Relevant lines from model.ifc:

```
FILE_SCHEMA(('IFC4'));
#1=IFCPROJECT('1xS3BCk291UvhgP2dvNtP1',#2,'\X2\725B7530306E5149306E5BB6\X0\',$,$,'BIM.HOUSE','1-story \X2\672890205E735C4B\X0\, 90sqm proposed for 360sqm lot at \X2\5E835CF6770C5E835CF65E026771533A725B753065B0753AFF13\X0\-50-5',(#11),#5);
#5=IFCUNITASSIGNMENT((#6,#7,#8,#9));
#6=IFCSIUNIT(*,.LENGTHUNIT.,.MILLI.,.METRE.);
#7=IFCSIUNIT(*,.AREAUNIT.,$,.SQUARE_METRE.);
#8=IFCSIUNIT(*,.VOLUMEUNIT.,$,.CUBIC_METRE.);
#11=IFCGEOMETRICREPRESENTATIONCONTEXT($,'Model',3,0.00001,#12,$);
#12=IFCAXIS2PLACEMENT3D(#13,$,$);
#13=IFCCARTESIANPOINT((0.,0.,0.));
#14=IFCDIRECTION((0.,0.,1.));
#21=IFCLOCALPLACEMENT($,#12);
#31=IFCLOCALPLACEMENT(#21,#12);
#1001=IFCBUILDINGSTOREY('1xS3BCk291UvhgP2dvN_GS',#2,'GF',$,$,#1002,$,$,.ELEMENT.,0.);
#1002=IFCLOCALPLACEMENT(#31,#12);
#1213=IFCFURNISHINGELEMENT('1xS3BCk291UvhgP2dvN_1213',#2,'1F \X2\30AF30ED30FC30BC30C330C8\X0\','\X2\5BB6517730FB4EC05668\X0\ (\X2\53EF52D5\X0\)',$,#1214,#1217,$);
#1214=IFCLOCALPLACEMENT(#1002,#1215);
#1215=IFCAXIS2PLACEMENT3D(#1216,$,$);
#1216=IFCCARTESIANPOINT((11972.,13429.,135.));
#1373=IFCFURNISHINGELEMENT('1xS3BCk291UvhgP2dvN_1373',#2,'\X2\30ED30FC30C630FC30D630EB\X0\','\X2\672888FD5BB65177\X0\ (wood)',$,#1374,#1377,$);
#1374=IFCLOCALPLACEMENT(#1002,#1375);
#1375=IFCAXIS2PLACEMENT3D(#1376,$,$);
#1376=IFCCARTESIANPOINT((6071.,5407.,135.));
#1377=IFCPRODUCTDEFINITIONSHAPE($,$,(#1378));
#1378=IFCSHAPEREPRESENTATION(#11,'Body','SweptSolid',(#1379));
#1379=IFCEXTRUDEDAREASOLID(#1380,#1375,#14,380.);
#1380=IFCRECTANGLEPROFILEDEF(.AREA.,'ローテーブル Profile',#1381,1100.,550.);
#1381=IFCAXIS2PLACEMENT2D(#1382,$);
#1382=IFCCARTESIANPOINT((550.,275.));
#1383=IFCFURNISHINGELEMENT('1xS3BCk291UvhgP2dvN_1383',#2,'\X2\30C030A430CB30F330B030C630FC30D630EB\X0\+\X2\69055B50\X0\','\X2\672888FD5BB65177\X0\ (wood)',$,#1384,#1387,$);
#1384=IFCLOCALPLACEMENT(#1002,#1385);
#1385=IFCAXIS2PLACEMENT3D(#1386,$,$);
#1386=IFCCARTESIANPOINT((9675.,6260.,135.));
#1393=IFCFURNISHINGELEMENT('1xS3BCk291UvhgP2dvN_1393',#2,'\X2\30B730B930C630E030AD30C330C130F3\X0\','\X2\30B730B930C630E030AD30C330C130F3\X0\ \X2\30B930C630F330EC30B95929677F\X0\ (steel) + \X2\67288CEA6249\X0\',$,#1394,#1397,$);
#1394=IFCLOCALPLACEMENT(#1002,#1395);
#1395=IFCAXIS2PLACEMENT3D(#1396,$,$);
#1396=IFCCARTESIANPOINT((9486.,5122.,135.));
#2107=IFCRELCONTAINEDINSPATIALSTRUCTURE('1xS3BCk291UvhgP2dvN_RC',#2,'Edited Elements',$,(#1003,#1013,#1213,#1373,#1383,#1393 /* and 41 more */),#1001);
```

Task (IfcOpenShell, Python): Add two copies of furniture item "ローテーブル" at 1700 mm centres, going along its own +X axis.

```python
import ifcopenshell
import ifcopenshell.api.geometry
import ifcopenshell.api.root
import ifcopenshell.util.element
import ifcopenshell.util.placement
import ifcopenshell.util.unit

model = ifcopenshell.open("model.ifc")
unit_scale = ifcopenshell.util.unit.calculate_unit_scale(model)


def reuse_history(source, copy):
    """copy_class also copies each property set's owner history, people and application; keep the originals."""
    for rel in copy.IsDefinedBy:
        if rel.is_a("IfcRelDefinesByProperties") and (history := rel.RelatingPropertyDefinition.OwnerHistory):
            rel.RelatingPropertyDefinition.OwnerHistory = source.OwnerHistory
            ifcopenshell.util.element.remove_deep2(model, history)


source = model.by_id(1373)
base = ifcopenshell.util.placement.get_local_placement(source.ObjectPlacement)
step = base[:3, 0] * 1.7 / unit_scale

for i in range(1, 3):
    copy = ifcopenshell.api.root.copy_class(model, product=source)
    copy.Representation = ifcopenshell.util.element.copy_deep(
        model, source.Representation, exclude=["IfcGeometricRepresentationContext", "IfcRepresentationMap"]
    )
    reuse_history(source, copy)
    matrix = base.copy()
    matrix[:3, 3] += i * step
    print("added at", matrix[:3, 3].round(3) + 0.0)
    ifcopenshell.api.geometry.edit_object_placement(model, product=copy, matrix=matrix, is_si=False)

model.write("model-out.ifc")
```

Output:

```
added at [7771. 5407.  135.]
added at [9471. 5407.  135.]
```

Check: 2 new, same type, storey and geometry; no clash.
